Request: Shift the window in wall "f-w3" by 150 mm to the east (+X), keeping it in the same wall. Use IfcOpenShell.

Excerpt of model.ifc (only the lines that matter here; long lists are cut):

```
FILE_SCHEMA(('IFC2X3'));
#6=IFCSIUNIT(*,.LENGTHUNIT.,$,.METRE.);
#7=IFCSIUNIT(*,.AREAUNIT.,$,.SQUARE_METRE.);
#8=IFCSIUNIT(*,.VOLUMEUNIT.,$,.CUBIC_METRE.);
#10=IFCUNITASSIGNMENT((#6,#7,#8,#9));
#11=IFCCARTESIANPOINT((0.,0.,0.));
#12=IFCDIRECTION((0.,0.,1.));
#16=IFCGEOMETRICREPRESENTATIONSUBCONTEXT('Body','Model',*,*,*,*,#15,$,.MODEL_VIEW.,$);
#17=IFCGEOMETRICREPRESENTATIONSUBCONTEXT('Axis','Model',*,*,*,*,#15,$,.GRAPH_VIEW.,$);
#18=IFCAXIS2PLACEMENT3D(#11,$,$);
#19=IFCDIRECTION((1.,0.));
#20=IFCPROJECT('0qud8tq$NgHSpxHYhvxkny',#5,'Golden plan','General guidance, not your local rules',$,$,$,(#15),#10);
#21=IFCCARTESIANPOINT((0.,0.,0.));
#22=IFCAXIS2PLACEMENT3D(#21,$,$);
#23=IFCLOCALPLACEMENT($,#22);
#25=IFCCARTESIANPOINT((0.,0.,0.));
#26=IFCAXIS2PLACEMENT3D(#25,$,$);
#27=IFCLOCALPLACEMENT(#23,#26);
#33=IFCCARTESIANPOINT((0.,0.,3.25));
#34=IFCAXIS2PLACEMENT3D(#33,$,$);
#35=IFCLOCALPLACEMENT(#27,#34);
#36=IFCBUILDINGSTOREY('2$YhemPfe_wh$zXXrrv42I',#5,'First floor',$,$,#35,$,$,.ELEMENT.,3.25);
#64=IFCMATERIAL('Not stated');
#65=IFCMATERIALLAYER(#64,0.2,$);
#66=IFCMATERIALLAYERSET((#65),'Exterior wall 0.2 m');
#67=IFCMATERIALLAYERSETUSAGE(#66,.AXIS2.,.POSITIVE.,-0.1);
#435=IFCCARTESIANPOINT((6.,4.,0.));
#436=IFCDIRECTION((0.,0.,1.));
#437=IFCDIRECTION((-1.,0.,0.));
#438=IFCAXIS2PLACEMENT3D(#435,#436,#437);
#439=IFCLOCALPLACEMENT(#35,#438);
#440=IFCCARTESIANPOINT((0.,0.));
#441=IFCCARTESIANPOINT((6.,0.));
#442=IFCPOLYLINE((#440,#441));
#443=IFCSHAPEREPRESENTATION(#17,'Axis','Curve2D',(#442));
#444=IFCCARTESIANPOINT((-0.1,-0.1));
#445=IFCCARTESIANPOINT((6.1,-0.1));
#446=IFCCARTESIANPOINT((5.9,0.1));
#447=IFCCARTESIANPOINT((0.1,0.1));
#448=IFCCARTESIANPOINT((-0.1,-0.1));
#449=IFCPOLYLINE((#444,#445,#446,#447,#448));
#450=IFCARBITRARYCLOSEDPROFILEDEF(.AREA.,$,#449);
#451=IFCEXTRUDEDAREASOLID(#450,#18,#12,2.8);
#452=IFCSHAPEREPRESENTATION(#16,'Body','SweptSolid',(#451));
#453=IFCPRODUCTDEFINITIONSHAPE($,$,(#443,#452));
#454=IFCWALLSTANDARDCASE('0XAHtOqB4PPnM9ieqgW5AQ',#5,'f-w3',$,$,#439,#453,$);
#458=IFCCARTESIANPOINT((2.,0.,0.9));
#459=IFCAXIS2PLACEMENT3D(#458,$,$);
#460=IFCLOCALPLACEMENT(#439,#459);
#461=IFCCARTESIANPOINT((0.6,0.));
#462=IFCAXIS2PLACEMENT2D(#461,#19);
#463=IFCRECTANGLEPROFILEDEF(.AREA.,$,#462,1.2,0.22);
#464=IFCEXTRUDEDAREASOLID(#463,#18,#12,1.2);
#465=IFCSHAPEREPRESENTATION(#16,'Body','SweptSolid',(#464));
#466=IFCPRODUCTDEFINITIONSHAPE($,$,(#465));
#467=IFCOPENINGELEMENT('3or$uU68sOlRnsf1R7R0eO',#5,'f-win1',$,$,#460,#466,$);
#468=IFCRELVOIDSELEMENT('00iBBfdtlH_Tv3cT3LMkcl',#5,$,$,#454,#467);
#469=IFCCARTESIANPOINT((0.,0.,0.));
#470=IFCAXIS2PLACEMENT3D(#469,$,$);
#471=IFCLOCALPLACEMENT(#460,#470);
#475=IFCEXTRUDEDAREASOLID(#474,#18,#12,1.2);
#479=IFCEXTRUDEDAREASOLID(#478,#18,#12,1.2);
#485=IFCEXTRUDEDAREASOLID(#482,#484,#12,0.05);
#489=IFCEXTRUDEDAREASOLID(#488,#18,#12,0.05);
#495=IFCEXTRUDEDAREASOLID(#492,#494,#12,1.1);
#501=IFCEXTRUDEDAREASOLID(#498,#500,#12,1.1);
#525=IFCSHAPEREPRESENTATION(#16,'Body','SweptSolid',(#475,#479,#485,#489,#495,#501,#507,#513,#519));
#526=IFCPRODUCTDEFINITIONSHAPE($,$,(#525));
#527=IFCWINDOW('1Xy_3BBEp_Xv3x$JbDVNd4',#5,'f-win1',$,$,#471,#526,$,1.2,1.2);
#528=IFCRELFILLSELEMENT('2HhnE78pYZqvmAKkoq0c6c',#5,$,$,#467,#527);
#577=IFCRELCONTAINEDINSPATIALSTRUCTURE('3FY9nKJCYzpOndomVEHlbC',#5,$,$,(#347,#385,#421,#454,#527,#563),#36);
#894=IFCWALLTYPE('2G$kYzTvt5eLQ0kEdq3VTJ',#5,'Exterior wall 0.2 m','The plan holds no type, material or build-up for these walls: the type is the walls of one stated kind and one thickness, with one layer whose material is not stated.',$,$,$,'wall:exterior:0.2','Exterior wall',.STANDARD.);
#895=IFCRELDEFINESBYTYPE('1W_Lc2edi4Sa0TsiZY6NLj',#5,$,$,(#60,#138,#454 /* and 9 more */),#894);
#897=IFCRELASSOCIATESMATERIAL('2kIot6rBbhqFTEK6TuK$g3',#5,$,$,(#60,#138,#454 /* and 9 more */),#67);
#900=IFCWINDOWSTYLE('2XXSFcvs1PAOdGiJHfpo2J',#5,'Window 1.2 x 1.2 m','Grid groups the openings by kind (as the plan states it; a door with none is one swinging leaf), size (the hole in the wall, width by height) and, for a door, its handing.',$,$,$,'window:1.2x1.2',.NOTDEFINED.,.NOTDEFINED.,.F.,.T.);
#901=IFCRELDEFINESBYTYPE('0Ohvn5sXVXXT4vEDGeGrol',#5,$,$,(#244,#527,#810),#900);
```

```python
import ifcopenshell
import ifcopenshell.api.geometry
import ifcopenshell.util.placement

model = ifcopenshell.open("model.ifc")

window = model.by_guid("1Xy_3BBEp_Xv3x$JbDVNd4")
opening = window.FillsVoids[0].RelatingOpeningElement
wall = opening.VoidsElements[0].RelatingBuildingElement

wall_matrix = ifcopenshell.util.placement.get_local_placement(wall.ObjectPlacement)
shift = wall_matrix[:3, 0] * -0.15
before = ifcopenshell.util.placement.get_local_placement(window.ObjectPlacement)[:3, 3].copy()

# The window is placed relative to its opening, so it follows when the opening moves.
matrix = ifcopenshell.util.placement.get_local_placement(opening.ObjectPlacement)
matrix[:3, 3] += shift
ifcopenshell.api.geometry.edit_object_placement(
    model, product=opening, matrix=matrix, is_si=False, should_transform_children=True
)

after = ifcopenshell.util.placement.get_local_placement(window.ObjectPlacement)[:3, 3]
print("window moved by", (after - before).round(3) + 0.0)

model.write("model_v2.ifc")
```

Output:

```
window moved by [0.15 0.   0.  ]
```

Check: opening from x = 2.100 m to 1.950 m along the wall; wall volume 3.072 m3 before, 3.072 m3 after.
